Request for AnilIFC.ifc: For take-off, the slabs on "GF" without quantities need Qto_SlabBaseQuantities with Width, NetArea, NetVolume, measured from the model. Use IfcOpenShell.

First a look at what the model holds.

```python
import ifcopenshell
import ifcopenshell.util.element
import ifcopenshell.util.unit

model = ifcopenshell.open("AnilIFC.ifc")
print(model.schema)
for unit_type in ("LENGTHUNIT", "AREAUNIT", "VOLUMEUNIT"):
    print(unit_type, ifcopenshell.util.unit.calculate_unit_scale(model, unit_type))
storey = next(s for s in model.by_type("IfcBuildingStorey") if s.Name == "GF")
slabs = [e for e in ifcopenshell.util.element.get_decomposition(storey) if e.is_a("IfcSlab")]
for e in sorted(slabs, key=lambda e: e.id()):
    print(e.id(), e.is_a(), e.Name, list(ifcopenshell.util.element.get_psets(e, qtos_only=True)), sep=" | ")
```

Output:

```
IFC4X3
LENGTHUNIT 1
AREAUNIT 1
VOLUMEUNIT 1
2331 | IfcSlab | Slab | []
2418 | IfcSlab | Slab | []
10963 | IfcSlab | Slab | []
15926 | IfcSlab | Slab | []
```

```python
import ifcopenshell
import ifcopenshell.api.pset
import ifcopenshell.geom
import ifcopenshell.util.element
import ifcopenshell.util.shape
import ifcopenshell.util.unit

model = ifcopenshell.open("AnilIFC.ifc")
unit_scale = ifcopenshell.util.unit.calculate_unit_scale(model)
area_scale = ifcopenshell.util.unit.calculate_unit_scale(model, "AREAUNIT")
volume_scale = ifcopenshell.util.unit.calculate_unit_scale(model, "VOLUMEUNIT")
settings = ifcopenshell.geom.settings()

storey = next(s for s in model.by_type("IfcBuildingStorey") if s.Name == "GF")
slabs = [e for e in ifcopenshell.util.element.get_decomposition(storey) if e.is_a("IfcSlab")]

for e in sorted(slabs, key=lambda e: e.id()):
    if ifcopenshell.util.element.get_psets(e, qtos_only=True, should_inherit=False):
        continue
    # Geometry comes back in metres, in the element's own axes.
    shape = ifcopenshell.geom.create_shape(settings, e)
    values = {
        "Width": ifcopenshell.util.shape.get_z(shape.geometry) / unit_scale,
        "NetArea": ifcopenshell.util.shape.get_footprint_area(shape.geometry) / area_scale,
        "NetVolume": ifcopenshell.util.shape.get_volume(shape.geometry) / volume_scale,
    }
    qto = ifcopenshell.api.pset.add_qto(model, product=e, name="Qto_SlabBaseQuantities")
    ifcopenshell.api.pset.edit_qto(model, qto=qto, properties=values)
    print(e.id(), {k: round(v, 3) for k, v in values.items()})

model.write("AnilIFC_rev.ifc")
```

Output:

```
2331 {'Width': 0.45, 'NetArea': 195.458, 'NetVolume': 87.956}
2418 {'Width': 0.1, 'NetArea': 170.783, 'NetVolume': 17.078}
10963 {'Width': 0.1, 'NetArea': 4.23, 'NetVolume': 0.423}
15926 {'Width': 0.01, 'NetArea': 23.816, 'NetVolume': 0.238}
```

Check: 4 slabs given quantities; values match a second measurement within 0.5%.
